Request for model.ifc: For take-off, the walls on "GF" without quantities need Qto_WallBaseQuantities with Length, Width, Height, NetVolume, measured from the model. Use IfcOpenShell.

First a look at what the model holds.

```python
import ifcopenshell
import ifcopenshell.util.element
import ifcopenshell.util.unit

model = ifcopenshell.open("model.ifc")
print(model.schema)
for unit_type in ("LENGTHUNIT", "AREAUNIT", "VOLUMEUNIT"):
    print(unit_type, ifcopenshell.util.unit.calculate_unit_scale(model, unit_type))
storey = next(s for s in model.by_type("IfcBuildingStorey") if s.Name == "GF")
walls = [e for e in ifcopenshell.util.element.get_decomposition(storey) if e.is_a("IfcWall")]
for e in sorted(walls, key=lambda e: e.id()):
    print(e.id(), e.is_a(), e.Name, list(ifcopenshell.util.element.get_psets(e, qtos_only=True)), sep=" | ")
```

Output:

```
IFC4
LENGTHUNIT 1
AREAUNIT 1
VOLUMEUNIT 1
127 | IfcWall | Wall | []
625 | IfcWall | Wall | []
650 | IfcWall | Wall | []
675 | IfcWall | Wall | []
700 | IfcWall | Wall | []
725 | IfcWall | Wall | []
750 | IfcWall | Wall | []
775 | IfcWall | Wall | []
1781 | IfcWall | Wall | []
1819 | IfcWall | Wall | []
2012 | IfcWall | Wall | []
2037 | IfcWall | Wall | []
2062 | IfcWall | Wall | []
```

```python
import ifcopenshell
import ifcopenshell.api.pset
import ifcopenshell.geom
import ifcopenshell.util.element
import ifcopenshell.util.shape
import ifcopenshell.util.unit

model = ifcopenshell.open("model.ifc")
unit_scale = ifcopenshell.util.unit.calculate_unit_scale(model)
volume_scale = ifcopenshell.util.unit.calculate_unit_scale(model, "VOLUMEUNIT")
settings = ifcopenshell.geom.settings()

storey = next(s for s in model.by_type("IfcBuildingStorey") if s.Name == "GF")
walls = [e for e in ifcopenshell.util.element.get_decomposition(storey) if e.is_a("IfcWall")]

for e in sorted(walls, key=lambda e: e.id()):
    if ifcopenshell.util.element.get_psets(e, qtos_only=True, should_inherit=False):
        continue
    # Geometry comes back in metres, in the element's own axes.
    shape = ifcopenshell.geom.create_shape(settings, e)
    values = {
        "Length": ifcopenshell.util.shape.get_x(shape.geometry) / unit_scale,
        "Width": ifcopenshell.util.shape.get_y(shape.geometry) / unit_scale,
        "Height": ifcopenshell.util.shape.get_z(shape.geometry) / unit_scale,
        "NetVolume": ifcopenshell.util.shape.get_volume(shape.geometry) / volume_scale,
    }
    qto = ifcopenshell.api.pset.add_qto(model, product=e, name="Qto_WallBaseQuantities")
    ifcopenshell.api.pset.edit_qto(model, qto=qto, properties=values)
    print(e.id(), {k: round(v, 3) for k, v in values.items()})

model.write("model_rev.ifc")
```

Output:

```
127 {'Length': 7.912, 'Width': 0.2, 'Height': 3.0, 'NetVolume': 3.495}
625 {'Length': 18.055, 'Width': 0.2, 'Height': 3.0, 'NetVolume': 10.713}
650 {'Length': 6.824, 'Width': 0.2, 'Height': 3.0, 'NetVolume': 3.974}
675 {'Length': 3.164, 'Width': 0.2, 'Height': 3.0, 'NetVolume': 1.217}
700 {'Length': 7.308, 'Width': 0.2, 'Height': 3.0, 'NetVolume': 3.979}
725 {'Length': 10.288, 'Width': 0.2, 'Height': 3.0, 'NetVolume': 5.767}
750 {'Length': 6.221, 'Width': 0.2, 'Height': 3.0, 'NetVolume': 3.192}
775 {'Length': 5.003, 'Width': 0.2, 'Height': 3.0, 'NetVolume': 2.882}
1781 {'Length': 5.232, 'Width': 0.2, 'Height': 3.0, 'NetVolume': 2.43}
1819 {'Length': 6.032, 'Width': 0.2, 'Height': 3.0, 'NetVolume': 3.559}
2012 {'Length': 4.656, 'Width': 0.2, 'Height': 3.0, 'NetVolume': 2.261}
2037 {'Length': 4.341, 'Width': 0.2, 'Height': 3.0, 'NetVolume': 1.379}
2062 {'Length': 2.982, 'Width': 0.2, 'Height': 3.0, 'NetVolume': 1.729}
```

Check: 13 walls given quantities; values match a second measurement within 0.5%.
